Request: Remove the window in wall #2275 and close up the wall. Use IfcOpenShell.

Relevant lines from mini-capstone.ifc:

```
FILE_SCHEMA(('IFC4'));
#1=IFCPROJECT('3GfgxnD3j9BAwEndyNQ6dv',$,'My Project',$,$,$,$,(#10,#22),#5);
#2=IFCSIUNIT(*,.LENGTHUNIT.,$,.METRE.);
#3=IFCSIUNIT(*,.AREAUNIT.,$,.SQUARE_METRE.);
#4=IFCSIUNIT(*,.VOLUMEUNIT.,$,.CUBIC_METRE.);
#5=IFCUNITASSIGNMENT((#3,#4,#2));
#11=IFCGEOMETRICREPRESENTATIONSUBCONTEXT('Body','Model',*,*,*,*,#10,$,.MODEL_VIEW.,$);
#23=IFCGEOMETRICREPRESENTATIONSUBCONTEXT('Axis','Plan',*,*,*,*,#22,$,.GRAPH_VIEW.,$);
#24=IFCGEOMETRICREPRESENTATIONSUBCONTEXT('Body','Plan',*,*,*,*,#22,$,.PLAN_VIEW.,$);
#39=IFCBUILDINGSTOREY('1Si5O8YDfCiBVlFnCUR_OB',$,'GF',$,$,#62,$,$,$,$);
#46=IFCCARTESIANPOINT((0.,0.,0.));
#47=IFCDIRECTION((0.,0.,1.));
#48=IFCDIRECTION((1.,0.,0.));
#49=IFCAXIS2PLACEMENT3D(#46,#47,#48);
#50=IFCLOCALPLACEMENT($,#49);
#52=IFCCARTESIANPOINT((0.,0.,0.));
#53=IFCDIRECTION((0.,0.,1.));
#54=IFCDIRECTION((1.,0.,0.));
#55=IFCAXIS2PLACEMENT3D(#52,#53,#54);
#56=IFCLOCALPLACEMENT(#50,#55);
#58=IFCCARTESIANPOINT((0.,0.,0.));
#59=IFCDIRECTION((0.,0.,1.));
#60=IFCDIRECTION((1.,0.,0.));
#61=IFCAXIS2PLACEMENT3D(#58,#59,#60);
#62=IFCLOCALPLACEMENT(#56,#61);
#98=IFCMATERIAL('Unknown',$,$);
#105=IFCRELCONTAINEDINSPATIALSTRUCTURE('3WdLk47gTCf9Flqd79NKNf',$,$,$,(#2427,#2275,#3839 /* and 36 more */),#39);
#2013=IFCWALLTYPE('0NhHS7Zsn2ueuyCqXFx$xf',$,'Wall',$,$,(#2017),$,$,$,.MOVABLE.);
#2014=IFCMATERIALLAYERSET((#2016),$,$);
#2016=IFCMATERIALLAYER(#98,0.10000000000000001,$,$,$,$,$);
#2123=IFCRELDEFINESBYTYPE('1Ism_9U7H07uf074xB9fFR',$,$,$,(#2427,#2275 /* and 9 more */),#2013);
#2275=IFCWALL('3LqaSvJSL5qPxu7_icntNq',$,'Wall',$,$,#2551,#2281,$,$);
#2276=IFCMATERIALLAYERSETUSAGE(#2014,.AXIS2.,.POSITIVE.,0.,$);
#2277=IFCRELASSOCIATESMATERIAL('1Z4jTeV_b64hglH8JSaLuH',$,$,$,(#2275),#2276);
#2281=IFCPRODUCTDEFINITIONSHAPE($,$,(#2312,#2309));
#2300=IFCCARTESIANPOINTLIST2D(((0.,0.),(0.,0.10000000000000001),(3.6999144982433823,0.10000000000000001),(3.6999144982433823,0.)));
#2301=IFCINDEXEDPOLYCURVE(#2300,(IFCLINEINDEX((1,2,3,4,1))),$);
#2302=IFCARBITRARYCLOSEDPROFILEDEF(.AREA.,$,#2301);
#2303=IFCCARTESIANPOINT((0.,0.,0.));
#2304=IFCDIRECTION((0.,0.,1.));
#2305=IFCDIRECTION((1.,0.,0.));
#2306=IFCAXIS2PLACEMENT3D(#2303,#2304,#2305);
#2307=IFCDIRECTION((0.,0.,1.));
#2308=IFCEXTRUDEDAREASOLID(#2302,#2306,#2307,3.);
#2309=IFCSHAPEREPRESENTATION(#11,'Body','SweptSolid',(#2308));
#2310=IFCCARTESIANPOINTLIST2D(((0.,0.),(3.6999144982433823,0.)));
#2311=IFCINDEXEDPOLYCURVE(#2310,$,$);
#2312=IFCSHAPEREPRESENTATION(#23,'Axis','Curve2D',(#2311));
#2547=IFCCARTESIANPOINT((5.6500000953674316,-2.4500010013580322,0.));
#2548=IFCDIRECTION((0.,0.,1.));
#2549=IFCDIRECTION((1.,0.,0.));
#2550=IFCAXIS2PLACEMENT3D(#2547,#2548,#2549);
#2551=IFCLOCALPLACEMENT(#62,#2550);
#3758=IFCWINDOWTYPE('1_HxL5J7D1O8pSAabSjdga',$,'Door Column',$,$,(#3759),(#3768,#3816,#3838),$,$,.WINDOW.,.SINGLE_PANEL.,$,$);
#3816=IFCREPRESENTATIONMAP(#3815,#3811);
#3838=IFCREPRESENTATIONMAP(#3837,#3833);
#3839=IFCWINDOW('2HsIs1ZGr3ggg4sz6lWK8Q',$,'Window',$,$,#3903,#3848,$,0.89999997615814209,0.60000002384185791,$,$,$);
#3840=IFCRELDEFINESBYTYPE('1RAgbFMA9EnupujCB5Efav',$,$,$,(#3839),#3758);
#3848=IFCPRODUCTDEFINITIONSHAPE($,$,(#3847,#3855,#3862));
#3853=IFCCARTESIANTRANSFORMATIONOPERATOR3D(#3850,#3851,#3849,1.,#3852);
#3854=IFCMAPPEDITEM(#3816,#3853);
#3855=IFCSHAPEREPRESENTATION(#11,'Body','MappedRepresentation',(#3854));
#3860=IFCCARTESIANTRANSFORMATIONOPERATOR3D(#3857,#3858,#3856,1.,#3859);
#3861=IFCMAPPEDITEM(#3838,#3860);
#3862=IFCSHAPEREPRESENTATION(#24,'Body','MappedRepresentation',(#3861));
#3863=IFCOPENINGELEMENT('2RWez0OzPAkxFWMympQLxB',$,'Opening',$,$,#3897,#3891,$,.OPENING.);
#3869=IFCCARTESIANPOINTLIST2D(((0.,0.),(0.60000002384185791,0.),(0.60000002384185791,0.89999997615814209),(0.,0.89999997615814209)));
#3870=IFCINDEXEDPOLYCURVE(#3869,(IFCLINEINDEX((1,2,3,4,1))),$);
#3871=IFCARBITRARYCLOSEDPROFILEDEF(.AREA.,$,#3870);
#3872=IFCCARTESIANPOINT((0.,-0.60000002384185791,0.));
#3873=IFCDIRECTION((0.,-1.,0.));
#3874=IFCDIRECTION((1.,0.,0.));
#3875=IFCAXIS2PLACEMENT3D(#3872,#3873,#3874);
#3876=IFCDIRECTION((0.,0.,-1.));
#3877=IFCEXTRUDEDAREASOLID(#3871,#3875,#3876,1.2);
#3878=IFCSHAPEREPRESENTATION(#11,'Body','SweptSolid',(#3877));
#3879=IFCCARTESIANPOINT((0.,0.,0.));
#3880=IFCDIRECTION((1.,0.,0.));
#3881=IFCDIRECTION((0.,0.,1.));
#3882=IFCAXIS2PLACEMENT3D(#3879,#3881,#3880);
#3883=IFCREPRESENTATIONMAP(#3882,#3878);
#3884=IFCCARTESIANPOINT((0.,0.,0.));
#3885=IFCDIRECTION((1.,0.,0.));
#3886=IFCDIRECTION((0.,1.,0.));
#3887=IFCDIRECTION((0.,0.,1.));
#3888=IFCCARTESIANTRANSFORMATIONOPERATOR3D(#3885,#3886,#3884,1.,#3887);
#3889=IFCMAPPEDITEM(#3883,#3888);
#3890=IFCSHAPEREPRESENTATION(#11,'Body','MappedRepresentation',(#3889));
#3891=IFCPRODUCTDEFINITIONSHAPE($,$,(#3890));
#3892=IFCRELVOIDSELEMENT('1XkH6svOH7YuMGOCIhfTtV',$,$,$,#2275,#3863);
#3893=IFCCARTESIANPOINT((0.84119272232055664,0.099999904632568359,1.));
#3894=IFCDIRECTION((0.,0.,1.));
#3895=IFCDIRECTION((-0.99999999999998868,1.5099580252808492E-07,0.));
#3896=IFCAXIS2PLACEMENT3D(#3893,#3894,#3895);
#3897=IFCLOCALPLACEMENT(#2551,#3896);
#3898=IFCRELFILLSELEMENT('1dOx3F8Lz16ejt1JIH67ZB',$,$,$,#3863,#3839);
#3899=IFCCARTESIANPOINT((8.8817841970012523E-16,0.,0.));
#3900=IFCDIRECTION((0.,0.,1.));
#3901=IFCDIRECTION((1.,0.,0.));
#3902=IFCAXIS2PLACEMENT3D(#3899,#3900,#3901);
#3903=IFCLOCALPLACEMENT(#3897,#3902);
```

```python
import ifcopenshell
import ifcopenshell.api.feature
import ifcopenshell.api.root
import ifcopenshell.geom
import ifcopenshell.util.shape

model = ifcopenshell.open("mini-capstone.ifc")
settings = ifcopenshell.geom.settings()


def volume(element):
    """Net volume in cubic metres, openings subtracted."""
    shape = ifcopenshell.geom.create_shape(settings, element)
    return ifcopenshell.util.shape.get_volume(shape.geometry)


window = model.by_guid("2HsIs1ZGr3ggg4sz6lWK8Q")
opening = window.FillsVoids[0].RelatingOpeningElement
wall = opening.VoidsElements[0].RelatingBuildingElement
before = volume(wall)

ifcopenshell.api.root.remove_product(model, product=window)
ifcopenshell.api.feature.remove_feature(model, feature=opening)

after = volume(wall)

print(f"wall volume {before:.3f} -> {after:.3f} m3")

model.write("mini-capstone_rev.ifc")
```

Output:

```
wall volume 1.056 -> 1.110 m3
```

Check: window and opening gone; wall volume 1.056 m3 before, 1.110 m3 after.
